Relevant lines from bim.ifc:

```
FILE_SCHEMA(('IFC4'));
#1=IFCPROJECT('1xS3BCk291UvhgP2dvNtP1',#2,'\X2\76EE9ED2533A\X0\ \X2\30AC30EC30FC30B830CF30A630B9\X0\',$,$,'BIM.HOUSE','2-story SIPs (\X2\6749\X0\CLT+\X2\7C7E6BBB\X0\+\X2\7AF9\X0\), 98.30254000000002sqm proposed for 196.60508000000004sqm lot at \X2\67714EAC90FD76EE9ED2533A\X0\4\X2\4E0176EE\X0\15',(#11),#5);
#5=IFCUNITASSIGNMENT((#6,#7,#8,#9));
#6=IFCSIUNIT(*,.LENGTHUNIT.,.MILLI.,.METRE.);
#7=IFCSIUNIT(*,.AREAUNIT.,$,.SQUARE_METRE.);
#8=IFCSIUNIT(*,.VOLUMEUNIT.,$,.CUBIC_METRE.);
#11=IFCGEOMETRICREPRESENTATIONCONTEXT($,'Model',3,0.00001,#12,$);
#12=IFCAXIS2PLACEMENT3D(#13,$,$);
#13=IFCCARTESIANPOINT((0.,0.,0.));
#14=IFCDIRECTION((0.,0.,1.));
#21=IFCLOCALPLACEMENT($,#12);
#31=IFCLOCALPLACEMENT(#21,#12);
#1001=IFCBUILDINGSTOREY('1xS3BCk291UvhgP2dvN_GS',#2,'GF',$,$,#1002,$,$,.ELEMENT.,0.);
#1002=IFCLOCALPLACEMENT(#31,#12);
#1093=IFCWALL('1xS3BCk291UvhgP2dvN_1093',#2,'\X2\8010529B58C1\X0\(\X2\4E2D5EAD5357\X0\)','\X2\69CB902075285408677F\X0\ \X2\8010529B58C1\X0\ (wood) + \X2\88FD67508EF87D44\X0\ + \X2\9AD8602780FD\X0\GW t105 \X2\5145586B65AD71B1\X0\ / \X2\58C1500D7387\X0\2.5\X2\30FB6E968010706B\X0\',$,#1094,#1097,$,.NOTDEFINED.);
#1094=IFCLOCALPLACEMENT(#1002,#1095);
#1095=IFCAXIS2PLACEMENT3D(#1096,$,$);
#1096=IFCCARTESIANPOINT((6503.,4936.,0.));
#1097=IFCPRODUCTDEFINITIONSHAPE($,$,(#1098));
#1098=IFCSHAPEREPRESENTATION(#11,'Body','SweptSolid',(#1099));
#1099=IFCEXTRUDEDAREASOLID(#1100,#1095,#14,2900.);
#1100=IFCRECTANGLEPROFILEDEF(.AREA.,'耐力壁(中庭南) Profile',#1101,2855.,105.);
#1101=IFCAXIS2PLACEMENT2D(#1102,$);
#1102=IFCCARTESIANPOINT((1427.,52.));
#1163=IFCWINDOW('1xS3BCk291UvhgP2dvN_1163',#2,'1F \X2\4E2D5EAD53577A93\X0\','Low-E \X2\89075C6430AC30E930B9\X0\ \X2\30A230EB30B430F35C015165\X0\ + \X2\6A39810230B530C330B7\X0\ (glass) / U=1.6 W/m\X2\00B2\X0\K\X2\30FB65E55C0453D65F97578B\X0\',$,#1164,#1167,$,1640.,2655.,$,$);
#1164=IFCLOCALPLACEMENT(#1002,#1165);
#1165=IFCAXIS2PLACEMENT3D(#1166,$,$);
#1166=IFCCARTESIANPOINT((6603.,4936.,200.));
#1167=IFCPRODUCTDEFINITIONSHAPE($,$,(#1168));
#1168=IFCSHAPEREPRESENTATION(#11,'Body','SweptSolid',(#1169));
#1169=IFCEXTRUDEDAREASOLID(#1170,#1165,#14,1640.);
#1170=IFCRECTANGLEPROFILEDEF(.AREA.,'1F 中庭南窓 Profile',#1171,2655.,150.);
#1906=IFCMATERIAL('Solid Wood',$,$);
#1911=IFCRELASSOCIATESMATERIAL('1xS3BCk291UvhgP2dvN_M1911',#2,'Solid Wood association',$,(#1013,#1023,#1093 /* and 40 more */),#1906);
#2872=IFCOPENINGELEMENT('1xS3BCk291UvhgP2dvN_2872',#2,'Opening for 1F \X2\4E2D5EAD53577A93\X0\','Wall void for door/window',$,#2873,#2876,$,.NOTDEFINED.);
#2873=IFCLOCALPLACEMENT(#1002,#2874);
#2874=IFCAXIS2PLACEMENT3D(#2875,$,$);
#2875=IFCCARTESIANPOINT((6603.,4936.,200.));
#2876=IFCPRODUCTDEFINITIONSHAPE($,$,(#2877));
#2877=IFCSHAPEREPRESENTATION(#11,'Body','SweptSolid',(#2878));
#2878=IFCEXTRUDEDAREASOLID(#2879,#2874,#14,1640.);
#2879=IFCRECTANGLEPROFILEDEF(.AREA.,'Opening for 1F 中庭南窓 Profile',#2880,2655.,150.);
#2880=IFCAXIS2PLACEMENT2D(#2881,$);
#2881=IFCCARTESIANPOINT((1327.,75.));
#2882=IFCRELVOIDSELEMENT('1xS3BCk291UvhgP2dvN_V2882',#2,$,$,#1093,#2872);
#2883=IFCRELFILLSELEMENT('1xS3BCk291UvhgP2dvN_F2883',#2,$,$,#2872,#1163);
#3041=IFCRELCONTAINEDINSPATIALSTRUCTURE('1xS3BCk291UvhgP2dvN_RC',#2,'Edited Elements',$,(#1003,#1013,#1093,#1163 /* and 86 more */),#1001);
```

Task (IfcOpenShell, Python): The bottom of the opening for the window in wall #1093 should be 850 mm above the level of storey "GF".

```python
import numpy as np
import ifcopenshell
import ifcopenshell.api.geometry
import ifcopenshell.geom
import ifcopenshell.util.element
import ifcopenshell.util.placement
import ifcopenshell.util.shape
import ifcopenshell.util.unit

model = ifcopenshell.open("bim.ifc")
unit_scale = ifcopenshell.util.unit.calculate_unit_scale(model)

window = model.by_guid("1xS3BCk291UvhgP2dvN_1163")
opening = window.FillsVoids[0].RelatingOpeningElement
storey = ifcopenshell.util.element.get_container(window, ifc_class="IfcBuildingStorey")
level = ifcopenshell.util.placement.get_local_placement(storey.ObjectPlacement)[2, 3]

# The opening's origin need not be at the sill, so measure its lowest point.
shape = ifcopenshell.geom.create_shape(ifcopenshell.geom.settings(), opening)
bottom = ifcopenshell.util.shape.get_shape_bottom_elevation(shape, shape.geometry) / unit_scale
dz = level + 850.0 - bottom

shift = np.array([0.0, 0.0, dz])
# The window is not placed relative to its opening, so move both.
for product in (opening, window):
    matrix = ifcopenshell.util.placement.get_local_placement(product.ObjectPlacement)
    matrix[:3, 3] += shift
    ifcopenshell.api.geometry.edit_object_placement(model, product=product, matrix=matrix, is_si=False)

print(f"moved by {dz * unit_scale:+.3f} m")

model.write("bim_edited.ifc")
```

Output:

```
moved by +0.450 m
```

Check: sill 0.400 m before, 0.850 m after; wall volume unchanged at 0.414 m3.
